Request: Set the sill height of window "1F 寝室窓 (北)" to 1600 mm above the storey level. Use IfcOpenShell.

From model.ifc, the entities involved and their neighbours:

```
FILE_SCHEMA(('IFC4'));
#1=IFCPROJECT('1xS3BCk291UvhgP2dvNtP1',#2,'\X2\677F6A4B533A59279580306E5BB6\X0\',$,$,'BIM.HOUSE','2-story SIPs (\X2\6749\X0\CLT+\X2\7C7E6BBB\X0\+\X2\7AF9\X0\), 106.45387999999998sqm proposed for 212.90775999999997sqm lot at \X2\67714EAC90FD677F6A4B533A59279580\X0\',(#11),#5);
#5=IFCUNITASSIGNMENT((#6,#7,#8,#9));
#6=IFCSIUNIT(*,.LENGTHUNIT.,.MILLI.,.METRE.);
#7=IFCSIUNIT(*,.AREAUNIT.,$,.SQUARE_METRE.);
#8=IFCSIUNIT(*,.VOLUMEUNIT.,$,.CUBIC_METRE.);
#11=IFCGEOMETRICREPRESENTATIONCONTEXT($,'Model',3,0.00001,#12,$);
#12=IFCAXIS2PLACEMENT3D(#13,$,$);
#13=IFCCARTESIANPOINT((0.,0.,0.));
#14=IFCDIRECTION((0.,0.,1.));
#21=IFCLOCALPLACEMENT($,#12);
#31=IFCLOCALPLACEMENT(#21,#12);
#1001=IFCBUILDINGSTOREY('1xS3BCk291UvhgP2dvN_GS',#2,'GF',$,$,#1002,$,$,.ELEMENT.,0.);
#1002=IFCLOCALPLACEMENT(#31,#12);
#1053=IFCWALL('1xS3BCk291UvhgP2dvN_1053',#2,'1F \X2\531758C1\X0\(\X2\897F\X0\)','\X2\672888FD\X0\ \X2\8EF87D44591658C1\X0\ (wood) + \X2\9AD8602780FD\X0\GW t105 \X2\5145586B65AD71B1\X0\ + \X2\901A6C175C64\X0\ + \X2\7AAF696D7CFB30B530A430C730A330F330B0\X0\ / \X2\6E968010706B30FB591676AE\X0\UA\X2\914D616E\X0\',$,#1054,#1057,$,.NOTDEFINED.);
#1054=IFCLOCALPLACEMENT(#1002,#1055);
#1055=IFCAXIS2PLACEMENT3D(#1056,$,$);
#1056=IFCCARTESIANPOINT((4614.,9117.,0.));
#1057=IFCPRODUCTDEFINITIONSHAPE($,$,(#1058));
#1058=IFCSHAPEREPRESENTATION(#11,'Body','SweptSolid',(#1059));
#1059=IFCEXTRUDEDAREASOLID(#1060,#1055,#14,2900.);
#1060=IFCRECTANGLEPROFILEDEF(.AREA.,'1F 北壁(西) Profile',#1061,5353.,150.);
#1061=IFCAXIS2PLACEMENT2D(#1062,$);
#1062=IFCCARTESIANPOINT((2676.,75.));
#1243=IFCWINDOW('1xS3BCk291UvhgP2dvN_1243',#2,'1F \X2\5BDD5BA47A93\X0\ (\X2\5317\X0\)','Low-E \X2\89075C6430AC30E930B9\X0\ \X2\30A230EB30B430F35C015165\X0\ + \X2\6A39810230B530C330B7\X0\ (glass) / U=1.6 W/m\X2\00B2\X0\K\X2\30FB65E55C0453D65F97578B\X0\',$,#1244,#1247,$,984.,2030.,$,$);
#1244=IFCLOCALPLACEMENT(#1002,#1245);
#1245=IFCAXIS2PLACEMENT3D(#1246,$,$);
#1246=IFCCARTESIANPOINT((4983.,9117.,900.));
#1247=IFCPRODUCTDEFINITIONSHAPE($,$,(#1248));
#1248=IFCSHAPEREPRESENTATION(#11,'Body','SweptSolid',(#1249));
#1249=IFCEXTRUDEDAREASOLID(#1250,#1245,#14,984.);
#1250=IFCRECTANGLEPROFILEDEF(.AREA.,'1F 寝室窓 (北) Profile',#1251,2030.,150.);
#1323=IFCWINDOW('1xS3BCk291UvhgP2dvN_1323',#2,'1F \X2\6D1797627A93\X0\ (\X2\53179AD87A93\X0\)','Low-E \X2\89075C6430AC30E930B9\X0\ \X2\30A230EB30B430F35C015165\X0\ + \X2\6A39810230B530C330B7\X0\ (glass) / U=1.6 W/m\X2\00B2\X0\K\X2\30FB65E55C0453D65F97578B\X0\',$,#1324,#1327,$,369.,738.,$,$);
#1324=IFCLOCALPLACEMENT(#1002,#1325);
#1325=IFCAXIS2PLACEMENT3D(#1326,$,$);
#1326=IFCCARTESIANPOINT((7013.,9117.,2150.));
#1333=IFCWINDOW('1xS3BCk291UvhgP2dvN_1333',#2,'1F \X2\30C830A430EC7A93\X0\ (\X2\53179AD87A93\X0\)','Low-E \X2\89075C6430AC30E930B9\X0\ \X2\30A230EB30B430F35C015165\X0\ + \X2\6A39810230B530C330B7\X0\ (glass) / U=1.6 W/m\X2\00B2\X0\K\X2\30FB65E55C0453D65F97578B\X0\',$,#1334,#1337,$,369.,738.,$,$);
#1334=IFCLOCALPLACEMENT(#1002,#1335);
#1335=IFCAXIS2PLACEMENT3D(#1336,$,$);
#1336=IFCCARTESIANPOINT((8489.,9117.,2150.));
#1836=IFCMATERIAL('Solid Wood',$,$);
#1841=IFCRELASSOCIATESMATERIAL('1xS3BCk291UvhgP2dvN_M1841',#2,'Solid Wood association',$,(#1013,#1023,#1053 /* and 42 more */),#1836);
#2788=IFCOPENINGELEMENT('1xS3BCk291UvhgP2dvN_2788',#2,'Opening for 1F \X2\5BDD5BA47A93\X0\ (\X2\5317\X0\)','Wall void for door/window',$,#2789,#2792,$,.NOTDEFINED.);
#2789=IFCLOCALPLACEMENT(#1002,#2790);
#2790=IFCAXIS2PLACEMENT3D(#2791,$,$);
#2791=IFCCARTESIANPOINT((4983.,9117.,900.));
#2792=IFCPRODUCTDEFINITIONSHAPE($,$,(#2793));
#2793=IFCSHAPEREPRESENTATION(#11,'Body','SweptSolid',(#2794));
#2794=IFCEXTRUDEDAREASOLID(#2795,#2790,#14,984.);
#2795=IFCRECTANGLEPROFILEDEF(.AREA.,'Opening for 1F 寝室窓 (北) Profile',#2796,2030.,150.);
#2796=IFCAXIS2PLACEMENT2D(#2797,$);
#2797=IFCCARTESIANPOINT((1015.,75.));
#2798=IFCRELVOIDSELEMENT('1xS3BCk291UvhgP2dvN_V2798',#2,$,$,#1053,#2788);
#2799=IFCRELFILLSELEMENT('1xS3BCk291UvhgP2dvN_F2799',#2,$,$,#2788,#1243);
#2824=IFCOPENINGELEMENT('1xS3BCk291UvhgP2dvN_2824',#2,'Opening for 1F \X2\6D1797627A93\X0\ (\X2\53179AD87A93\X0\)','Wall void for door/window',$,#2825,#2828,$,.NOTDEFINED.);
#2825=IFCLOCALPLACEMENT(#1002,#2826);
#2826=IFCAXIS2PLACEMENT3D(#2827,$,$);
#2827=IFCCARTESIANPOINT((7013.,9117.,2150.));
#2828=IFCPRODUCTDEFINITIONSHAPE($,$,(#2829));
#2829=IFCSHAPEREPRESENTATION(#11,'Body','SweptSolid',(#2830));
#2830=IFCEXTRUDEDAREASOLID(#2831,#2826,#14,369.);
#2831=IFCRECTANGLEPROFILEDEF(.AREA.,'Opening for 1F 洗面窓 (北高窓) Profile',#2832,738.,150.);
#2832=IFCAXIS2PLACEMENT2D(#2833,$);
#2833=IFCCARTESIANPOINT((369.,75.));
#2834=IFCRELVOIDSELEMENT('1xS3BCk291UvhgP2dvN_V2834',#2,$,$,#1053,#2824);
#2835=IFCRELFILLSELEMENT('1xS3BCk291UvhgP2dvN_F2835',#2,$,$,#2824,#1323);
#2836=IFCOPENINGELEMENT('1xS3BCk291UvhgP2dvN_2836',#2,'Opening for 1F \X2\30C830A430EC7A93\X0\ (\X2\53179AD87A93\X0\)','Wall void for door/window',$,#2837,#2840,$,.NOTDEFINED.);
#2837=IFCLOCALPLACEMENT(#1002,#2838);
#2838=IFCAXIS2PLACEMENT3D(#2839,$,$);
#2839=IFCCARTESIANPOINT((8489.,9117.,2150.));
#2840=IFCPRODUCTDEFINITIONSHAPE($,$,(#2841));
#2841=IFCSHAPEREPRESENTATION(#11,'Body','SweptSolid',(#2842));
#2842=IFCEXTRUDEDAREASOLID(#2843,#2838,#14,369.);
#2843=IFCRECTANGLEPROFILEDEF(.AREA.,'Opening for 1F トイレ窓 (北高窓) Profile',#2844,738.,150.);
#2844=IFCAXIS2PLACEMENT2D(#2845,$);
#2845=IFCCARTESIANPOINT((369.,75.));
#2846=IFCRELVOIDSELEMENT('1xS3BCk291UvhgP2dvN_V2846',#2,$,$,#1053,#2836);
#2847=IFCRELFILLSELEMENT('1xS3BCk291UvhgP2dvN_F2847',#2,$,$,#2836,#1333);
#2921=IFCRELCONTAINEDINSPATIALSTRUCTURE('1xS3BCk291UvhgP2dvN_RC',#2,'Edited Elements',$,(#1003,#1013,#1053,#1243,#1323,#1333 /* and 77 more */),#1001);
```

```python
import numpy as np
import ifcopenshell
import ifcopenshell.api.geometry
import ifcopenshell.geom
import ifcopenshell.util.element
import ifcopenshell.util.placement
import ifcopenshell.util.shape
import ifcopenshell.util.unit

model = ifcopenshell.open("model.ifc")
unit_scale = ifcopenshell.util.unit.calculate_unit_scale(model)

window = model.by_guid("1xS3BCk291UvhgP2dvN_1243")
opening = window.FillsVoids[0].RelatingOpeningElement
storey = ifcopenshell.util.element.get_container(window, ifc_class="IfcBuildingStorey")
level = ifcopenshell.util.placement.get_local_placement(storey.ObjectPlacement)[2, 3]

# The opening's origin need not be at the sill, so measure its lowest point.
shape = ifcopenshell.geom.create_shape(ifcopenshell.geom.settings(), opening)
bottom = ifcopenshell.util.shape.get_shape_bottom_elevation(shape, shape.geometry) / unit_scale
dz = level + 1600.0 - bottom

shift = np.array([0.0, 0.0, dz])
# The window is not placed relative to its opening, so move both.
for product in (opening, window):
    matrix = ifcopenshell.util.placement.get_local_placement(product.ObjectPlacement)
    matrix[:3, 3] += shift
    ifcopenshell.api.geometry.edit_object_placement(model, product=product, matrix=matrix, is_si=False)

print(f"moved by {dz * unit_scale:+.3f} m")

model.write("model_updated.ifc")
```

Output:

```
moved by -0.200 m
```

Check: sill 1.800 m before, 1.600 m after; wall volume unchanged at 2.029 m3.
